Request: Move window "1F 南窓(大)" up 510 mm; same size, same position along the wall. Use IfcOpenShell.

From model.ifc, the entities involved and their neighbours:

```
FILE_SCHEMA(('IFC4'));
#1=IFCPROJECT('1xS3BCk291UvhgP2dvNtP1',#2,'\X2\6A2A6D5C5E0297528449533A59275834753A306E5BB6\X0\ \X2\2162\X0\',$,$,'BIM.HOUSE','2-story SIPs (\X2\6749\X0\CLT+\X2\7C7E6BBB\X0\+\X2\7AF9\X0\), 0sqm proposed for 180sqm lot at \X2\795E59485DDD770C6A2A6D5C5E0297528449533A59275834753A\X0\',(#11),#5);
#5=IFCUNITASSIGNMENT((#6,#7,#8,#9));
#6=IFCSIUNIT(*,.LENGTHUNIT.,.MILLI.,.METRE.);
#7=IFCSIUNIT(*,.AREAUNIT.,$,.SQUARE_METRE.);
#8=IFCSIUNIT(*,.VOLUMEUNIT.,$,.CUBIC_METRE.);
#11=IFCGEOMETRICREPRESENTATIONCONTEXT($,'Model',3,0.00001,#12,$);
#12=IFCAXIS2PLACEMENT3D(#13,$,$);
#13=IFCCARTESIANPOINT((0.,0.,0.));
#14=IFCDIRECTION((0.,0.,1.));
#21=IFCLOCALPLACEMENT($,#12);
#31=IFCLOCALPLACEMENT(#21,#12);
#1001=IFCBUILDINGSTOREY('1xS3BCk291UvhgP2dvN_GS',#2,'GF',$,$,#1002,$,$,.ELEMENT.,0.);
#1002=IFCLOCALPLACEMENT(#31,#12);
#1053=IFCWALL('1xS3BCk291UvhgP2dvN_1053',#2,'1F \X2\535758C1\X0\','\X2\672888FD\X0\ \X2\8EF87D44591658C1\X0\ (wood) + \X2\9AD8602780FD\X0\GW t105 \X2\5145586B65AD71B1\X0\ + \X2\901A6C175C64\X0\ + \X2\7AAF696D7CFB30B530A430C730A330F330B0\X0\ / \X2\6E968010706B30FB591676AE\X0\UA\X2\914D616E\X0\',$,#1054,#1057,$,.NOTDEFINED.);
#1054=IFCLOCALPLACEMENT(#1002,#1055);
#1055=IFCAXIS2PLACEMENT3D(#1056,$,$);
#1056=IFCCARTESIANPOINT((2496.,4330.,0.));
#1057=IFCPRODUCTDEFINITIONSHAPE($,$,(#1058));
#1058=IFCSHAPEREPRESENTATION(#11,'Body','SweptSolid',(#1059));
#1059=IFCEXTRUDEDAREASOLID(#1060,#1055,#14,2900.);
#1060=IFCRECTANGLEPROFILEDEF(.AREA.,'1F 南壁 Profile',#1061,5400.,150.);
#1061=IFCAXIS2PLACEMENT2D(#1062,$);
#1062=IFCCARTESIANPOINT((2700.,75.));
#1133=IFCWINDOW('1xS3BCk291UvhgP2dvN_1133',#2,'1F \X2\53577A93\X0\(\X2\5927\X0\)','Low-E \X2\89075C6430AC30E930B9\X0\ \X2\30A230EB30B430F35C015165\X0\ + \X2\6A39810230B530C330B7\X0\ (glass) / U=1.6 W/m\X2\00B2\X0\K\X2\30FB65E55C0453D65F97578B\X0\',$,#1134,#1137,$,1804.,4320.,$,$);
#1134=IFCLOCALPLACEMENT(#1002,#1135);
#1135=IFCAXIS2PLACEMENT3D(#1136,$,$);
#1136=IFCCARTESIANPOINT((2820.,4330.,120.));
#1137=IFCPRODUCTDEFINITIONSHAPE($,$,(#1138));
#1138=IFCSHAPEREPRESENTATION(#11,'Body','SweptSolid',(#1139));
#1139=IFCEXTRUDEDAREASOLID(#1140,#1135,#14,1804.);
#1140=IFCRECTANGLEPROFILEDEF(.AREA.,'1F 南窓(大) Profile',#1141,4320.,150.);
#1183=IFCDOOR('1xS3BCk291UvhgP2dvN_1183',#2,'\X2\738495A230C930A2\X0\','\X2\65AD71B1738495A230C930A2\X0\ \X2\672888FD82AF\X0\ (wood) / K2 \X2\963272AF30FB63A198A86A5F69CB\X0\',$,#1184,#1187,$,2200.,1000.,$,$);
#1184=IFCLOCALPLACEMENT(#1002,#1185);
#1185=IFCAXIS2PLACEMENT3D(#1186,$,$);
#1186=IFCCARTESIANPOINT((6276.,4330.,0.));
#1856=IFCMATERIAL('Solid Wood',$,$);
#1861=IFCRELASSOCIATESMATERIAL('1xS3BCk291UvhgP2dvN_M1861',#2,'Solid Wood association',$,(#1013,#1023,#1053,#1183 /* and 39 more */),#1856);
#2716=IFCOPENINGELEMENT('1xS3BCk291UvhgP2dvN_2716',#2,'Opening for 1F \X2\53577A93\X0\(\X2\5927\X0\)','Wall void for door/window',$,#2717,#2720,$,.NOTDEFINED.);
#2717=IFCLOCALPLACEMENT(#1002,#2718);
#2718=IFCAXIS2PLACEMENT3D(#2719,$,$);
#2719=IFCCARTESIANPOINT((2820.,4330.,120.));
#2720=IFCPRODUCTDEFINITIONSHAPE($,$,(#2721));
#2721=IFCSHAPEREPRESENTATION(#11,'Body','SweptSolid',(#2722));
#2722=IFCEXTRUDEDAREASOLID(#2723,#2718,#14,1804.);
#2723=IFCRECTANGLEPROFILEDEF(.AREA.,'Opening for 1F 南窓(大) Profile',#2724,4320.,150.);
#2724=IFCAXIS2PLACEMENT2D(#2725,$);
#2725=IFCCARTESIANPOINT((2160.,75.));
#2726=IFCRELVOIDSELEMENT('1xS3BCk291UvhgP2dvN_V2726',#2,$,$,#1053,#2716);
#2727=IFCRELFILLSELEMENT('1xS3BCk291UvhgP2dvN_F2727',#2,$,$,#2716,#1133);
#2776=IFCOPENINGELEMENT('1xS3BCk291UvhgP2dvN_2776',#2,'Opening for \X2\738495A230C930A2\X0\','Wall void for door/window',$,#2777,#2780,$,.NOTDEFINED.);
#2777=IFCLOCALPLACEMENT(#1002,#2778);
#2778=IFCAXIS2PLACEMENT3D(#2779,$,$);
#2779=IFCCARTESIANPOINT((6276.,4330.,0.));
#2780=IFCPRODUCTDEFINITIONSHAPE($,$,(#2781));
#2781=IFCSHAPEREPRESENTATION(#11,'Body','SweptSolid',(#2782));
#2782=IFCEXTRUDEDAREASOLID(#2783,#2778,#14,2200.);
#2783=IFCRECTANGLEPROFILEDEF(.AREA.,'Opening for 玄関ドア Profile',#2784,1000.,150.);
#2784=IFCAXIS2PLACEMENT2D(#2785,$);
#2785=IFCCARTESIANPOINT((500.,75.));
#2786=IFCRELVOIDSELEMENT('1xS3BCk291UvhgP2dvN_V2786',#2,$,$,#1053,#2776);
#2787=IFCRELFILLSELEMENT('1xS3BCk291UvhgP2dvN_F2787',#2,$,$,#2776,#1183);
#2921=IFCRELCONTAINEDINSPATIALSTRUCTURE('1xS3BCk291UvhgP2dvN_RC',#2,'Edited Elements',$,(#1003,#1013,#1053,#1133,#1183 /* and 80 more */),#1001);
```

```python
import numpy as np
import ifcopenshell
import ifcopenshell.api.geometry
import ifcopenshell.util.placement
import ifcopenshell.util.unit

model = ifcopenshell.open("model.ifc")
unit_scale = ifcopenshell.util.unit.calculate_unit_scale(model)

window = model.by_id(1133)
opening = window.FillsVoids[0].RelatingOpeningElement
dz = 0.51 / unit_scale

shift = np.array([0.0, 0.0, dz])
# The window is not placed relative to its opening, so move both.
for product in (opening, window):
    matrix = ifcopenshell.util.placement.get_local_placement(product.ObjectPlacement)
    matrix[:3, 3] += shift
    ifcopenshell.api.geometry.edit_object_placement(model, product=product, matrix=matrix, is_si=False)

print(f"moved by {dz * unit_scale:+.3f} m")

model.write("model-out.ifc")
```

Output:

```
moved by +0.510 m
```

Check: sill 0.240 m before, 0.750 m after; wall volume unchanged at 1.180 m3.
